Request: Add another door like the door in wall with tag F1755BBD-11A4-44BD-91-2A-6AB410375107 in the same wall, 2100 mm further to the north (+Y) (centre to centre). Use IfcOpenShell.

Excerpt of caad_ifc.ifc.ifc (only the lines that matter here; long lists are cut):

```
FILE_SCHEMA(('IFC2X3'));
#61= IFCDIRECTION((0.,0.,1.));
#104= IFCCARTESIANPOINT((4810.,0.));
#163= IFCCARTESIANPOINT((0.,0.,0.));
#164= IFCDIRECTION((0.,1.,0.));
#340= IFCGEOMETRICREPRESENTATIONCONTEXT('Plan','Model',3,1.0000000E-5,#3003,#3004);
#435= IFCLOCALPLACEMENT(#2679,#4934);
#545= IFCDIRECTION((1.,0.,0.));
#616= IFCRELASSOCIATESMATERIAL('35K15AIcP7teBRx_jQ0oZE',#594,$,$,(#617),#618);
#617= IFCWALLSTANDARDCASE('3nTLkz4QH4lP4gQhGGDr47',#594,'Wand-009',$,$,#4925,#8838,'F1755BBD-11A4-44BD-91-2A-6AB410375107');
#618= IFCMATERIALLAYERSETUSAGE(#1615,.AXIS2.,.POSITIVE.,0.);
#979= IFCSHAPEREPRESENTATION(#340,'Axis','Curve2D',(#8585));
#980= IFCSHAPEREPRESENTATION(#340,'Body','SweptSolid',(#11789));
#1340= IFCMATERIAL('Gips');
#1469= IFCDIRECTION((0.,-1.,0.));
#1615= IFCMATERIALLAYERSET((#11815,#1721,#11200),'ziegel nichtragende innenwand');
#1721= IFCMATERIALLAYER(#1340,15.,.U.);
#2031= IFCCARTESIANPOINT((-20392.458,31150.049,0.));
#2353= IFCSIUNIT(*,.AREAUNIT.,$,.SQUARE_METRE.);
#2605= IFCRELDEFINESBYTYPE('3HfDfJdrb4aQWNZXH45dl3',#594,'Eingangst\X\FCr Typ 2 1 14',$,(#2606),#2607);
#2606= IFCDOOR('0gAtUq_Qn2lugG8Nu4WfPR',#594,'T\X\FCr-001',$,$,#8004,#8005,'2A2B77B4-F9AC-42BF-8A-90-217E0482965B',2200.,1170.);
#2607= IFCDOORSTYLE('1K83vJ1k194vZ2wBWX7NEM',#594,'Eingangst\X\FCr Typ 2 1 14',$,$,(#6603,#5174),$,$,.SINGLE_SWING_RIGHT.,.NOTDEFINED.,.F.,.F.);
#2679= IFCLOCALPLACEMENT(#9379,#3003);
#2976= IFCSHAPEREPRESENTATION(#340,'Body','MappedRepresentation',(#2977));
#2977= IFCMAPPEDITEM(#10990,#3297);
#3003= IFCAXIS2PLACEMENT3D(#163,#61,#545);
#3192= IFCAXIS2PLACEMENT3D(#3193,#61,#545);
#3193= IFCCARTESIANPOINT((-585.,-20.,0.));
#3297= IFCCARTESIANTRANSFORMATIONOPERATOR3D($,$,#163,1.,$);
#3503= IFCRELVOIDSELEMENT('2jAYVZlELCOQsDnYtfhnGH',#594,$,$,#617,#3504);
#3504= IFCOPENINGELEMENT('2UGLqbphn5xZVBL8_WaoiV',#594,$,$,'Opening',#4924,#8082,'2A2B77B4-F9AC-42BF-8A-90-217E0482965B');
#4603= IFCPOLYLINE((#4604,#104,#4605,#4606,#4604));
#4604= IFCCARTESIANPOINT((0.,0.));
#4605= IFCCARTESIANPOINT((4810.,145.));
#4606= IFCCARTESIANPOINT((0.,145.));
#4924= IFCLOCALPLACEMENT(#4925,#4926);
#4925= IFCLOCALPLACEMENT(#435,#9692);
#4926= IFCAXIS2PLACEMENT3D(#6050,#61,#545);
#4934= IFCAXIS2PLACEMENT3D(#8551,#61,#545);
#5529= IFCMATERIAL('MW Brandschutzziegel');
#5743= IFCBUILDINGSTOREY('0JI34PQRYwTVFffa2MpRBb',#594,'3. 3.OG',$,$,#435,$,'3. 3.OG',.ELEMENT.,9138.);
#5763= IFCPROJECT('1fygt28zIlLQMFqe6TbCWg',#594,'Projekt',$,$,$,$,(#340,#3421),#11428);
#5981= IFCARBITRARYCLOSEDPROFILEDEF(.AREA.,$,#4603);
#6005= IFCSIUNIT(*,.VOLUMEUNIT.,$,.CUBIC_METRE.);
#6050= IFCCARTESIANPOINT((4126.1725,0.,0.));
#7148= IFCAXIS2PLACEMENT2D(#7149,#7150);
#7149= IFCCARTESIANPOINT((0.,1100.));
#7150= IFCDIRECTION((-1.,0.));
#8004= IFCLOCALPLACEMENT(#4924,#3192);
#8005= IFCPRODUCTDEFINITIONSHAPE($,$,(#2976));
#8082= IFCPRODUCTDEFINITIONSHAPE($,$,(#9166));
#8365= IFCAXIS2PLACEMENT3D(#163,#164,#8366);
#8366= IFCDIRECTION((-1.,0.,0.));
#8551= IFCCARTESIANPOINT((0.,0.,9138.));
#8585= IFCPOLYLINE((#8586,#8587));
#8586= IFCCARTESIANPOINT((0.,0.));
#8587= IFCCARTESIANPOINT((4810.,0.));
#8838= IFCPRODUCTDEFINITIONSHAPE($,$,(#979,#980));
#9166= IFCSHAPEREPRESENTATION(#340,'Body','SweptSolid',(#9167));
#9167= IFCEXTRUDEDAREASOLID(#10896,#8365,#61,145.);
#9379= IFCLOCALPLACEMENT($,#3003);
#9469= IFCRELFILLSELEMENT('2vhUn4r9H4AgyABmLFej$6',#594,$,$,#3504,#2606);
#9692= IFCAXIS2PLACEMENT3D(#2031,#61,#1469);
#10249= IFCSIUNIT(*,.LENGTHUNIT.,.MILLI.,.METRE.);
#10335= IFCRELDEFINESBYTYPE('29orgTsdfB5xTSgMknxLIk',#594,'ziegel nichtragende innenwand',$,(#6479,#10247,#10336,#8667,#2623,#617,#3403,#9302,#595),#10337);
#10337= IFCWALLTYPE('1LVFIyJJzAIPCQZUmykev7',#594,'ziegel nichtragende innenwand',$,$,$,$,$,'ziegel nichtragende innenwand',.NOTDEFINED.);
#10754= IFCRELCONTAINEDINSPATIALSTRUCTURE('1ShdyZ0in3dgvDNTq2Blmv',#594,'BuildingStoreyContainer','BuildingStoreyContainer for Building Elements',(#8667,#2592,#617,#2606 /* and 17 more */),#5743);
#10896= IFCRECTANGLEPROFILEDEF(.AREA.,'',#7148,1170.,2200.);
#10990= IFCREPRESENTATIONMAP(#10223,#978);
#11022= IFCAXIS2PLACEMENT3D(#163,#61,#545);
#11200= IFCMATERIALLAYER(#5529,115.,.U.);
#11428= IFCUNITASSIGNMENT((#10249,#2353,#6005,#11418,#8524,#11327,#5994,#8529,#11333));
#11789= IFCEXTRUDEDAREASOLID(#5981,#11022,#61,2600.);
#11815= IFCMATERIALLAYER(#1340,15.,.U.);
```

```python
import ifcopenshell
import ifcopenshell.api.feature
import ifcopenshell.api.geometry
import ifcopenshell.api.root
import ifcopenshell.geom
import ifcopenshell.util.element
import ifcopenshell.util.placement
import ifcopenshell.util.shape
import ifcopenshell.util.unit

model = ifcopenshell.open("caad_ifc.ifc.ifc")
unit_scale = ifcopenshell.util.unit.calculate_unit_scale(model)
settings = ifcopenshell.geom.settings()


def volume(element):
    """Net volume in cubic metres, openings subtracted."""
    shape = ifcopenshell.geom.create_shape(settings, element)
    return ifcopenshell.util.shape.get_volume(shape.geometry)


door = model.by_guid("0gAtUq_Qn2lugG8Nu4WfPR")
opening = door.FillsVoids[0].RelatingOpeningElement
wall = opening.VoidsElements[0].RelatingBuildingElement
before = volume(wall)
shift = ifcopenshell.util.placement.get_local_placement(wall.ObjectPlacement)[:3, 0] * -2.1 / unit_scale

# copy_class copies the void relationship, type, container and properties, but no geometry.
new_opening = ifcopenshell.api.root.copy_class(model, product=opening)
new_opening.Representation = ifcopenshell.util.element.copy_deep(
    model, opening.Representation, exclude=["IfcGeometricRepresentationContext", "IfcRepresentationMap"]
)
new_opening.Tag = None
new_door = ifcopenshell.api.root.copy_class(model, product=door)
new_door.Representation = ifcopenshell.util.element.copy_deep(
    model, door.Representation, exclude=["IfcGeometricRepresentationContext", "IfcRepresentationMap"]
)
new_door.Tag = None
fills = ifcopenshell.api.feature.add_filling(model, opening=new_opening, element=new_door)
fills.OwnerHistory = new_door.OwnerHistory  # required in IFC2X3

for old, new in ((opening, new_opening), (door, new_door)):
    matrix = ifcopenshell.util.placement.get_local_placement(old.ObjectPlacement)
    matrix[:3, 3] += shift
    ifcopenshell.api.geometry.edit_object_placement(model, product=new, matrix=matrix, is_si=False)

after = volume(wall)

print(f"wall volume {before:.3f} -> {after:.3f} m3")

model.write("caad_ifc.ifc_rev.ifc")
```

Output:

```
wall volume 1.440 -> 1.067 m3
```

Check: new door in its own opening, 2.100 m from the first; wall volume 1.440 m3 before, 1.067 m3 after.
